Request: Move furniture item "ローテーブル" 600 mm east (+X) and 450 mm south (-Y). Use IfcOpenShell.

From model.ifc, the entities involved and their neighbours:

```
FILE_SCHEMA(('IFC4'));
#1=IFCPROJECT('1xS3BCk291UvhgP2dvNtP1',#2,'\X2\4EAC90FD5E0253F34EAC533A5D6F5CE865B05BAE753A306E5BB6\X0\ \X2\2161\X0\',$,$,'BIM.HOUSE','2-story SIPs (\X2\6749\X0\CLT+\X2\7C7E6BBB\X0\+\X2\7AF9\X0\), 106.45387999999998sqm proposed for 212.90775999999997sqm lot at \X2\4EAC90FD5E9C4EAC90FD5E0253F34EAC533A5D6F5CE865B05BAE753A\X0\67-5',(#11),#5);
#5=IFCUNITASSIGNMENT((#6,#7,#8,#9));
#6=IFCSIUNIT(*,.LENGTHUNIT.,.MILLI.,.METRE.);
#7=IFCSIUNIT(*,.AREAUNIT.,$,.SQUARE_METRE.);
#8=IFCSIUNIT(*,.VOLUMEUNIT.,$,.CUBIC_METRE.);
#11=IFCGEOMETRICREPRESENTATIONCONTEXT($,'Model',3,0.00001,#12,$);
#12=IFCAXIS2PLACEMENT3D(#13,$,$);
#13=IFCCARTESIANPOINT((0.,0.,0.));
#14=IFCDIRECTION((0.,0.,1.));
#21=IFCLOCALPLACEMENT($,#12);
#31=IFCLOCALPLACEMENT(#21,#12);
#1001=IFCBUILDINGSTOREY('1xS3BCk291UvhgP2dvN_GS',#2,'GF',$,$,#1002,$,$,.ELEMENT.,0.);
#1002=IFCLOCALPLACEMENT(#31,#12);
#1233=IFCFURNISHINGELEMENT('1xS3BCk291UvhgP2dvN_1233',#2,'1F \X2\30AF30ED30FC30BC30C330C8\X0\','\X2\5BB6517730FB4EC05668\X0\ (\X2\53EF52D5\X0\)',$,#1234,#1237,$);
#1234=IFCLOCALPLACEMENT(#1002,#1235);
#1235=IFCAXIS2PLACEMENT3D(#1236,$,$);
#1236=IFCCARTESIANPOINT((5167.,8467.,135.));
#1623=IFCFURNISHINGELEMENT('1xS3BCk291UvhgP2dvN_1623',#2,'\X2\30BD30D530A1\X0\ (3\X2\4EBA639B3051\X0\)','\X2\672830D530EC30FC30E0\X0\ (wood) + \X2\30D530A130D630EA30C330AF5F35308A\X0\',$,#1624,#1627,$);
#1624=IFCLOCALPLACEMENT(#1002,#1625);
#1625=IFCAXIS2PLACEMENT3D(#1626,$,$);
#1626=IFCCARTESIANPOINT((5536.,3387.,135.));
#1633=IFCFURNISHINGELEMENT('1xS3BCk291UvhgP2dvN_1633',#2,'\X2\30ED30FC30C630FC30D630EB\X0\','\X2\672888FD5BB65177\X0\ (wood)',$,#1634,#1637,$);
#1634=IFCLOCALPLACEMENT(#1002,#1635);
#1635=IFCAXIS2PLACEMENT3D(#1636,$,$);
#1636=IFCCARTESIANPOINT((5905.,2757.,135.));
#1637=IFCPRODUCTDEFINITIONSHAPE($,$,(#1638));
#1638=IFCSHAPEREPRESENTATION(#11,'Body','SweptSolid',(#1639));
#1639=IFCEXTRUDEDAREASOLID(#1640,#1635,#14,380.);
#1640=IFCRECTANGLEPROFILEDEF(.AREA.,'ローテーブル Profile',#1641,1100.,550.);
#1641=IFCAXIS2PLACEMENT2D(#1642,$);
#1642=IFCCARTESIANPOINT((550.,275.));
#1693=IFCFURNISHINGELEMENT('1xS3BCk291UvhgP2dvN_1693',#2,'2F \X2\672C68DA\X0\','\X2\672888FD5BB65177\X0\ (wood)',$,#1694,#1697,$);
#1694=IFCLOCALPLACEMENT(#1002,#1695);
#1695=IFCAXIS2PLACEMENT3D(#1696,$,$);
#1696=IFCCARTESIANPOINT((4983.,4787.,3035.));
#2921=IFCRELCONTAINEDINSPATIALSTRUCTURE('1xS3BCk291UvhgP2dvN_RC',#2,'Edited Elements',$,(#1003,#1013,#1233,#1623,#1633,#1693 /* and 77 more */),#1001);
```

```python
import ifcopenshell
import ifcopenshell.api.geometry
import ifcopenshell.util.placement
import ifcopenshell.util.unit

model = ifcopenshell.open("model.ifc")
unit_scale = ifcopenshell.util.unit.calculate_unit_scale(model)

item = model.by_guid("1xS3BCk291UvhgP2dvN_1633")
matrix = ifcopenshell.util.placement.get_local_placement(item.ObjectPlacement)
matrix[0, 3] += 0.6 / unit_scale
matrix[1, 3] -= 0.45 / unit_scale
ifcopenshell.api.geometry.edit_object_placement(model, product=item, matrix=matrix, is_si=False)

print(ifcopenshell.util.placement.get_local_placement(item.ObjectPlacement).round(3) + 0.0)

model.write("model_edited.ifc")
```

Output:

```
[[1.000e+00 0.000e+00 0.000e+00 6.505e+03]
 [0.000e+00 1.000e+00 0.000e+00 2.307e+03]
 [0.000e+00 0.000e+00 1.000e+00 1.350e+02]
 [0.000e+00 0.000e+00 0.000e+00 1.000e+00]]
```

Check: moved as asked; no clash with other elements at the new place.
